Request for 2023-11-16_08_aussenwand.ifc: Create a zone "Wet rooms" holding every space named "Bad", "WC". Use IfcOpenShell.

First a look at what the model holds.

```python
import ifcopenshell

model = ifcopenshell.open("2023-11-16_08_aussenwand.ifc")
print(model.schema)
seen = {}
for space in model.by_type("IfcSpace"):
    seen[space.LongName] = seen.get(space.LongName, 0) + 1
for name, count in sorted(seen.items(), key=str):
    print(count, "x", name)
print("zones:", [z.Name for z in model.by_type("IfcZone")][:20])
```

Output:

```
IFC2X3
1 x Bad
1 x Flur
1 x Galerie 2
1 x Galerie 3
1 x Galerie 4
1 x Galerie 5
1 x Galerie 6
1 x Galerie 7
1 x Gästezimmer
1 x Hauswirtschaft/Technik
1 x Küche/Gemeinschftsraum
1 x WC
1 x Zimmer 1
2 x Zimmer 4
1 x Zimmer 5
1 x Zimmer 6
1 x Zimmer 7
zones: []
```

```python
import ifcopenshell
import ifcopenshell.api.group
import ifcopenshell.api.root

model = ifcopenshell.open("2023-11-16_08_aussenwand.ifc")

names = {"Bad", "WC"}
spaces = [s for s in model.by_type("IfcSpace") if s.LongName in names]

zone = ifcopenshell.api.root.create_entity(model, ifc_class="IfcZone", name="Wet rooms")
ifcopenshell.api.group.assign_group(model, products=spaces, group=zone)
print(len(spaces), "spaces in", zone.Name)

model.write("2023-11-16_08_aussenwand_v2.ifc")
```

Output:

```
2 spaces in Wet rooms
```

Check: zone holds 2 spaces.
